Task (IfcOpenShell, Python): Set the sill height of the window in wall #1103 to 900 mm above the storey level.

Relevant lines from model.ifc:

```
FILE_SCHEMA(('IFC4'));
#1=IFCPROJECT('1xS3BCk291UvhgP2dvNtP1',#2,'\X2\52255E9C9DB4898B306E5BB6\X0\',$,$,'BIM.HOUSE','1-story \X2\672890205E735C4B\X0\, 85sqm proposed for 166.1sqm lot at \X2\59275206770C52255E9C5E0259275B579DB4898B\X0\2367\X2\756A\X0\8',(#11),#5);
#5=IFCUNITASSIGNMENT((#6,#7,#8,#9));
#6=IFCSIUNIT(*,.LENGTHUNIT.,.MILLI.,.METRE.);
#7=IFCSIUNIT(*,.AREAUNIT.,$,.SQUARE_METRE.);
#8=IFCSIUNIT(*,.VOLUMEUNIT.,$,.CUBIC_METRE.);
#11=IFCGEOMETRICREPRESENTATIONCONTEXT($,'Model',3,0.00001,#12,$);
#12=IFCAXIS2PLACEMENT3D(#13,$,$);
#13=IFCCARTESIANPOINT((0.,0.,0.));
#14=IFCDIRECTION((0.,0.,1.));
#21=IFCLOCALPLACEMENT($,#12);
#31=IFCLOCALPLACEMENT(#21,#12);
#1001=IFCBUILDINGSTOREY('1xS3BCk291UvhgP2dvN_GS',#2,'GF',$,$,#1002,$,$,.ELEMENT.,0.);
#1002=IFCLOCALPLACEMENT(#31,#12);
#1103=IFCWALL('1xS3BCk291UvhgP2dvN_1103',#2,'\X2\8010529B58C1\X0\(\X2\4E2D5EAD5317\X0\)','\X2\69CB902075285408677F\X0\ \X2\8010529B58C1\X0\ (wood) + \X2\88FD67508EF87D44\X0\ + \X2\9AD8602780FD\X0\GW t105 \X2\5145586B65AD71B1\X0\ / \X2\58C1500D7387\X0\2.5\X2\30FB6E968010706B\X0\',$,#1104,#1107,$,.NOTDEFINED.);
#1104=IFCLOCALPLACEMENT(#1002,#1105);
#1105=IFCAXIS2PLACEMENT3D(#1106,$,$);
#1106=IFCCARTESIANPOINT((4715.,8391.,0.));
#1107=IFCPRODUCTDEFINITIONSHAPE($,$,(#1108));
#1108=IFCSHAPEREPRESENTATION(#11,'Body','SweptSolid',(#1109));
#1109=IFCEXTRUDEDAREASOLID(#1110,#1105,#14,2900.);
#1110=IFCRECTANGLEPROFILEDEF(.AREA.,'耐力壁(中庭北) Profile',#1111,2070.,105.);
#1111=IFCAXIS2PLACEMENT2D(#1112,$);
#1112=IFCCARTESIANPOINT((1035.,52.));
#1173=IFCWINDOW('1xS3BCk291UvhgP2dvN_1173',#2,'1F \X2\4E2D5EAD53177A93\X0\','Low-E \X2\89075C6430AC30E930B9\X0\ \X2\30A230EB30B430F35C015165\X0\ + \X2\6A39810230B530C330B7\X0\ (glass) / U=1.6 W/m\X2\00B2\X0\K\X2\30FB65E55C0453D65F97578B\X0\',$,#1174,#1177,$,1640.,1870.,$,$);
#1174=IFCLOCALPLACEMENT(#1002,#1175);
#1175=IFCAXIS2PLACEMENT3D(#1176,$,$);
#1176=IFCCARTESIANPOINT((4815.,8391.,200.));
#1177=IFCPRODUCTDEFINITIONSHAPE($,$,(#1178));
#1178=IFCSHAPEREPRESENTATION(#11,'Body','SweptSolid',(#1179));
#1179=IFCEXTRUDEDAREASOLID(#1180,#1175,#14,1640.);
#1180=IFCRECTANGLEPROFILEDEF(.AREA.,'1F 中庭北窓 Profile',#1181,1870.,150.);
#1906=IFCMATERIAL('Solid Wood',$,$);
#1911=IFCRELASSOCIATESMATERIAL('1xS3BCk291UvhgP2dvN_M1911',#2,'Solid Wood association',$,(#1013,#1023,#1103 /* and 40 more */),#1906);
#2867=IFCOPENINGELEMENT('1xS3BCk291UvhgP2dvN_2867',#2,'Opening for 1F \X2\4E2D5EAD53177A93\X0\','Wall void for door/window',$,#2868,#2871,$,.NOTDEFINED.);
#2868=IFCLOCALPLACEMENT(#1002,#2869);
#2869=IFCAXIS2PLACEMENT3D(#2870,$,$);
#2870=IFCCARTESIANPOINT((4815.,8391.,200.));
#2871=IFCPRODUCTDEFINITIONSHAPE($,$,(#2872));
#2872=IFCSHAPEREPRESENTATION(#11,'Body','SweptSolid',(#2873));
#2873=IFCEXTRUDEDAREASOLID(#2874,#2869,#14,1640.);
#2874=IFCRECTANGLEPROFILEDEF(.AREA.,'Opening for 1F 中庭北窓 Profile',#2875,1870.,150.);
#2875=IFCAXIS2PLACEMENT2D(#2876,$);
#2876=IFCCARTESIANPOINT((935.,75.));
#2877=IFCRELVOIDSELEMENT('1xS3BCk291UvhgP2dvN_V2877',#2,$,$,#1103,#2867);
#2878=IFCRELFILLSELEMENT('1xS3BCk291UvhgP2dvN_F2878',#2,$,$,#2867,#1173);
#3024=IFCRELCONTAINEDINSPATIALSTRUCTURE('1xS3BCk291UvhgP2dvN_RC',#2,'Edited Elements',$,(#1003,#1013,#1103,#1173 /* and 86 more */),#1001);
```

```python
import numpy as np
import ifcopenshell
import ifcopenshell.api.geometry
import ifcopenshell.geom
import ifcopenshell.util.element
import ifcopenshell.util.placement
import ifcopenshell.util.shape
import ifcopenshell.util.unit

model = ifcopenshell.open("model.ifc")
unit_scale = ifcopenshell.util.unit.calculate_unit_scale(model)

window = model.by_guid("1xS3BCk291UvhgP2dvN_1173")
opening = window.FillsVoids[0].RelatingOpeningElement
storey = ifcopenshell.util.element.get_container(window, ifc_class="IfcBuildingStorey")
level = ifcopenshell.util.placement.get_local_placement(storey.ObjectPlacement)[2, 3]

# The opening's origin need not be at the sill, so measure its lowest point.
shape = ifcopenshell.geom.create_shape(ifcopenshell.geom.settings(), opening)
bottom = ifcopenshell.util.shape.get_shape_bottom_elevation(shape, shape.geometry) / unit_scale
dz = level + 900.0 - bottom

shift = np.array([0.0, 0.0, dz])
# The window is not placed relative to its opening, so move both.
for product in (opening, window):
    matrix = ifcopenshell.util.placement.get_local_placement(product.ObjectPlacement)
    matrix[:3, 3] += shift
    ifcopenshell.api.geometry.edit_object_placement(model, product=product, matrix=matrix, is_si=False)

print(f"moved by {dz * unit_scale:+.3f} m")

model.write("model_rev.ifc")
```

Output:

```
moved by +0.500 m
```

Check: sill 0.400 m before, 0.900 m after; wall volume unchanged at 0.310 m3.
